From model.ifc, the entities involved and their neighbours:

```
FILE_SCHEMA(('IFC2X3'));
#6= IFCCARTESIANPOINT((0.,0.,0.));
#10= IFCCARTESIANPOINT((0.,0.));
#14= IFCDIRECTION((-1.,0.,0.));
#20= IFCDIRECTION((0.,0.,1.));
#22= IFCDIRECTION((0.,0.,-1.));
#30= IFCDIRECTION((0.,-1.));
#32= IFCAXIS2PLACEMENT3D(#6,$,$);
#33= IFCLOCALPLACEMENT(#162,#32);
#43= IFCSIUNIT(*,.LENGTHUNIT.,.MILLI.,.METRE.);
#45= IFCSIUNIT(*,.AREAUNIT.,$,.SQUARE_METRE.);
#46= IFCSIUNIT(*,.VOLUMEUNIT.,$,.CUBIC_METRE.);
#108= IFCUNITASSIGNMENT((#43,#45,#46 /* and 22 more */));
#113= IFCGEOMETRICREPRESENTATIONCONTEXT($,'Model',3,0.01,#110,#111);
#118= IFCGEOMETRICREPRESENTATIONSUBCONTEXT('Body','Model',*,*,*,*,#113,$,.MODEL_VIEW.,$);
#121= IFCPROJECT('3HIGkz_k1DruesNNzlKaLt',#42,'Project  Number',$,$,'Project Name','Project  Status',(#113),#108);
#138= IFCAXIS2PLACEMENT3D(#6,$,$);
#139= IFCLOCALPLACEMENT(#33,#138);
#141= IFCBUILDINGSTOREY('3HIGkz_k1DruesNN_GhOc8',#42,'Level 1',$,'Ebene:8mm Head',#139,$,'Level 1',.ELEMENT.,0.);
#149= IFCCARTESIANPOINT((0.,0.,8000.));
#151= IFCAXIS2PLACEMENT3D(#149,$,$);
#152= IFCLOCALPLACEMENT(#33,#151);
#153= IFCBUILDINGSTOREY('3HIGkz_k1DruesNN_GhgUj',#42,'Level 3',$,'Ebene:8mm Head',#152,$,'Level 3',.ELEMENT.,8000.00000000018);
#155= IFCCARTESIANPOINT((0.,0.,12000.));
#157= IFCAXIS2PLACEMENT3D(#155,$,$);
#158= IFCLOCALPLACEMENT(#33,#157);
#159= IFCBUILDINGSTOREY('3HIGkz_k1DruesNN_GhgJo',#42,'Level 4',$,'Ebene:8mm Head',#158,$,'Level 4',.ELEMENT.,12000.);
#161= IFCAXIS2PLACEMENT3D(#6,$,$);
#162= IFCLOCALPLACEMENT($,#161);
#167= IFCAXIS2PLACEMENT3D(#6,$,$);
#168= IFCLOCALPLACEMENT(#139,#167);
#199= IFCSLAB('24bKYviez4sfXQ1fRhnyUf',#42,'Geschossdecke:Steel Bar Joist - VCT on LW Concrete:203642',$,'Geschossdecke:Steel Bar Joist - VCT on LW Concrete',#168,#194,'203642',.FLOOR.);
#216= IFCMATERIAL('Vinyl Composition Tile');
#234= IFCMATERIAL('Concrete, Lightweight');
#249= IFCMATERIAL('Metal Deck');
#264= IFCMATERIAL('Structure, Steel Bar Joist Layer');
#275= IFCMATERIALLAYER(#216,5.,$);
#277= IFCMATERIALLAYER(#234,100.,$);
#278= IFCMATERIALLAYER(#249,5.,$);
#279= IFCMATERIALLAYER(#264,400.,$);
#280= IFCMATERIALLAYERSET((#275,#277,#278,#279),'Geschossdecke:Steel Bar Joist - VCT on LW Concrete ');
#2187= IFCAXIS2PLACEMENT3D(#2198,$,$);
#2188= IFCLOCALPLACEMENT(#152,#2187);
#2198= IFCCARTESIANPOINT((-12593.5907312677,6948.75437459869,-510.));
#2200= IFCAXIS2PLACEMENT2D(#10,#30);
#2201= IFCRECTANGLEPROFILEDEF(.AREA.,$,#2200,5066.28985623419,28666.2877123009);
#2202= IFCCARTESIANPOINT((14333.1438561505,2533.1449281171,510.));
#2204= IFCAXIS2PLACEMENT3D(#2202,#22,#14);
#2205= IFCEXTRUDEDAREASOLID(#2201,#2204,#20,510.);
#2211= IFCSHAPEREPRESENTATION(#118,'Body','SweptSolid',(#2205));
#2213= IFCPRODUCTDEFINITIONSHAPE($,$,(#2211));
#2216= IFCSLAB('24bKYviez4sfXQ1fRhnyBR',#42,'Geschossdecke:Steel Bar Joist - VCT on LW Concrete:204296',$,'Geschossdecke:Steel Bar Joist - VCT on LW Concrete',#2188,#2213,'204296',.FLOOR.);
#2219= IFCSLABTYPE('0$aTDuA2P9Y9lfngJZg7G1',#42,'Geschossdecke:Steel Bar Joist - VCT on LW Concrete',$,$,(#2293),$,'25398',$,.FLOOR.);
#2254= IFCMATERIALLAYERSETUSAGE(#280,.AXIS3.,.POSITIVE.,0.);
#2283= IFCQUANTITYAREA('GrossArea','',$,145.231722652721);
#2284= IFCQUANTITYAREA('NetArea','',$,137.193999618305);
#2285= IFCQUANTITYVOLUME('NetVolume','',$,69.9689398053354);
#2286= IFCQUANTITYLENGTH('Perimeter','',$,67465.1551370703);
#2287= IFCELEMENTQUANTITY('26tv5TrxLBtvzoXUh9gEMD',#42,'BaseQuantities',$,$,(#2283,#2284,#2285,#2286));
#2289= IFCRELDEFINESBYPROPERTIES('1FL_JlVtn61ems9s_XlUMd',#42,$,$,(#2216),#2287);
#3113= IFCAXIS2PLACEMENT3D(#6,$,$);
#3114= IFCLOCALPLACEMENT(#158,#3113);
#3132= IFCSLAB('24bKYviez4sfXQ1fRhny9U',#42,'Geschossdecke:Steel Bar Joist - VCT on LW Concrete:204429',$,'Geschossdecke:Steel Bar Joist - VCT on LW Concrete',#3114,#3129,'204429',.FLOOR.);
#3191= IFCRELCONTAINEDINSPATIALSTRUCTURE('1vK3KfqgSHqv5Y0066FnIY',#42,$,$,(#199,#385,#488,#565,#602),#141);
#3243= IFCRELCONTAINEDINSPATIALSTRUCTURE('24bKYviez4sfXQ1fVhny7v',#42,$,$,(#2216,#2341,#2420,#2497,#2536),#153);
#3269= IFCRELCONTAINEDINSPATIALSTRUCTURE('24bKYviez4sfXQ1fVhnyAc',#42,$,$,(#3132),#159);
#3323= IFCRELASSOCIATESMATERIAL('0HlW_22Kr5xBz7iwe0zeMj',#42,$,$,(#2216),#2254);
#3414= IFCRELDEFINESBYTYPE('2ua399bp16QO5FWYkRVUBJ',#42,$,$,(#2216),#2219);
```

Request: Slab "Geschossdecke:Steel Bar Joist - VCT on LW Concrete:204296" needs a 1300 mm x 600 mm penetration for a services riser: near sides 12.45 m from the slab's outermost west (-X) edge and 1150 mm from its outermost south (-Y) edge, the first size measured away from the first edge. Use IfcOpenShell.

```python
import numpy as np
import ifcopenshell
import ifcopenshell.api.feature
import ifcopenshell.api.geometry
import ifcopenshell.api.pset
import ifcopenshell.api.root
import ifcopenshell.geom
import ifcopenshell.util.element
import ifcopenshell.util.placement
import ifcopenshell.util.representation
import ifcopenshell.util.shape
import ifcopenshell.util.unit

model = ifcopenshell.open("model.ifc")
unit_scale = ifcopenshell.util.unit.calculate_unit_scale(model)
area_scale = ifcopenshell.util.unit.calculate_unit_scale(model, "AREAUNIT")
volume_scale = ifcopenshell.util.unit.calculate_unit_scale(model, "VOLUMEUNIT")
settings = ifcopenshell.geom.settings()


def volume(element):
    """Net volume in cubic metres, openings subtracted."""
    shape = ifcopenshell.geom.create_shape(settings, element)
    return ifcopenshell.util.shape.get_volume(shape.geometry)


slab = model.by_guid("24bKYviez4sfXQ1fRhnyBR")
before = volume(slab)

# Extent in the slab's own axes, in metres. The edges named are its -X and -Y sides.
slab_shape = ifcopenshell.geom.create_shape(settings, slab)
vertices = ifcopenshell.util.shape.get_vertices(slab_shape.geometry)
x_min, y_min, bottom = vertices.min(axis=0)
top = vertices[:, 2].max()

opening = ifcopenshell.api.root.create_entity(model, ifc_class="IfcOpeningElement", name="Services riser opening")
context = ifcopenshell.util.representation.get_context(model, "Model", "Body", "MODEL_VIEW")
width, depth = 1.3, 0.6
outline = [(0.0, 0.0), (width, 0.0), (width, depth), (0.0, depth), (0.0, 0.0)]
# Overshoot both faces by 50 mm so the cut is clean.
shape = ifcopenshell.api.geometry.add_slab_representation(
    model, context=context, depth=top - bottom + 0.1, polyline=outline
)
ifcopenshell.api.geometry.assign_representation(model, product=opening, representation=shape)

matrix = ifcopenshell.util.placement.get_local_placement(slab.ObjectPlacement)
matrix[:, 3] = matrix @ np.append(np.array([x_min + 12.45, y_min + 1.15, bottom - 0.05]) / unit_scale, 1.0)
ifcopenshell.api.geometry.edit_object_placement(model, product=opening, matrix=matrix, is_si=False)
ifcopenshell.api.feature.add_feature(model, feature=opening, element=slab)

after = volume(slab)

# Update the slab's stored quantities.
qto = model.by_id(ifcopenshell.util.element.get_pset(slab, "BaseQuantities", should_inherit=False)["id"])
ifcopenshell.api.pset.edit_qto(model, qto=qto, properties={
    "NetArea": after / (top - bottom) / area_scale,
    "NetVolume": after / volume_scale,
})

print(f"slab volume {before:.3f} -> {after:.3f} m3")

model.write("model-out.ifc")
```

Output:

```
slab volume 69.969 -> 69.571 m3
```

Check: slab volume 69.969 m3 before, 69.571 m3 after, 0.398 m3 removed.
